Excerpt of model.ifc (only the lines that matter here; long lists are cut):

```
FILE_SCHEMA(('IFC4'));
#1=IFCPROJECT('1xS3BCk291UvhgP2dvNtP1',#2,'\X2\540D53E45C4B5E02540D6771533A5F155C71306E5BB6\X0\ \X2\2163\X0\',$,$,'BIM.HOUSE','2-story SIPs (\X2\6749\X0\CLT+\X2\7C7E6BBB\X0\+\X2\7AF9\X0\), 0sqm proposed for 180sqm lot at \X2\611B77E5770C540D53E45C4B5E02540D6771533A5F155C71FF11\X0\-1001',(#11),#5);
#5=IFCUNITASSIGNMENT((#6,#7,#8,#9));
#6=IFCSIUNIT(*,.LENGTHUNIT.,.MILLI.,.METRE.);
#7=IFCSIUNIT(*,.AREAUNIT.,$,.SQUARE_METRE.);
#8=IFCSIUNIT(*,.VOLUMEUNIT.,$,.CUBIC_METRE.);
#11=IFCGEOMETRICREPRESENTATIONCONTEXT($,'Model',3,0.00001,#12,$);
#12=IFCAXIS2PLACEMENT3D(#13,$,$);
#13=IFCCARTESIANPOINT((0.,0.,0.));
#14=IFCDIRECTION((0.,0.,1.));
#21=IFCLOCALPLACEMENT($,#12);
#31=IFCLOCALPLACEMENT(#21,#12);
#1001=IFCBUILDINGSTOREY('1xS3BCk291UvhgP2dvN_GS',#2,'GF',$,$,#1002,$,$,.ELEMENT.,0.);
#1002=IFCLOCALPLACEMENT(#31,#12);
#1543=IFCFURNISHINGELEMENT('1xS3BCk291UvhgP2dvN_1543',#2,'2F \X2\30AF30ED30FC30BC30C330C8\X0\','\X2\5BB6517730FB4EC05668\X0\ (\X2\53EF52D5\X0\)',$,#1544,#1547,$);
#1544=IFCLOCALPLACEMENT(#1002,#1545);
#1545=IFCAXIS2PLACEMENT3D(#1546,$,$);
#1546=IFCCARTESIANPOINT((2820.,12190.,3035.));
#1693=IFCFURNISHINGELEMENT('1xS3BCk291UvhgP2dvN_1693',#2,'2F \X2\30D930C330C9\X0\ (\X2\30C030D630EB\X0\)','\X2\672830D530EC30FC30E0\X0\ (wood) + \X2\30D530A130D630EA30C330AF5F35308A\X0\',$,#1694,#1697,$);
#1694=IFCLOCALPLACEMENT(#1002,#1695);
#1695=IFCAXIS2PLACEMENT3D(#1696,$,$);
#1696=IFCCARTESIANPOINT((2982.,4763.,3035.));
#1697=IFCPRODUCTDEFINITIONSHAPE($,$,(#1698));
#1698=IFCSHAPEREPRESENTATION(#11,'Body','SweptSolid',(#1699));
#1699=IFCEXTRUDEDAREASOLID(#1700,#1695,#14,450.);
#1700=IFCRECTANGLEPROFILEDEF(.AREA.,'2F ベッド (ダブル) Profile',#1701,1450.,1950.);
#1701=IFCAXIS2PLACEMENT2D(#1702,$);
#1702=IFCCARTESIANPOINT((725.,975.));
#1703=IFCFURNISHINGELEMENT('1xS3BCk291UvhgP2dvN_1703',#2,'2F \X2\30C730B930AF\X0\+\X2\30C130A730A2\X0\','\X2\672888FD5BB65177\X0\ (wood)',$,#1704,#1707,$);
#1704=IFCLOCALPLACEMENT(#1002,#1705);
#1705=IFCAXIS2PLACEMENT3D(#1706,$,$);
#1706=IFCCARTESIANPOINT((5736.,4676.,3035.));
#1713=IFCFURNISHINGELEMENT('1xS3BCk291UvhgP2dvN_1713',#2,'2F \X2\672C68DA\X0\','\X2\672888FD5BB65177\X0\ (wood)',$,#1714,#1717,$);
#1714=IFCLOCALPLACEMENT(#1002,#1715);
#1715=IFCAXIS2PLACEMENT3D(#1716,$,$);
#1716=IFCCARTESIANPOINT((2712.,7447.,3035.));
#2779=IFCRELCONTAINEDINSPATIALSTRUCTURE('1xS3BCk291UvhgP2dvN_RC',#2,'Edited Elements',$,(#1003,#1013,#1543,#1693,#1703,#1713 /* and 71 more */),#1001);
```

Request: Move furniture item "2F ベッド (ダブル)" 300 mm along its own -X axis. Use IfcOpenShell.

```python
import ifcopenshell
import ifcopenshell.api.geometry
import ifcopenshell.util.placement

model = ifcopenshell.open("model.ifc")

item = model.by_guid("1xS3BCk291UvhgP2dvN_1693")
matrix = ifcopenshell.util.placement.get_local_placement(item.ObjectPlacement)
matrix[:3, 3] -= matrix[:3, 0] * 300.0
ifcopenshell.api.geometry.edit_object_placement(model, product=item, matrix=matrix, is_si=False)

print(ifcopenshell.util.placement.get_local_placement(item.ObjectPlacement).round(3) + 0.0)

model.write("model_updated.ifc")
```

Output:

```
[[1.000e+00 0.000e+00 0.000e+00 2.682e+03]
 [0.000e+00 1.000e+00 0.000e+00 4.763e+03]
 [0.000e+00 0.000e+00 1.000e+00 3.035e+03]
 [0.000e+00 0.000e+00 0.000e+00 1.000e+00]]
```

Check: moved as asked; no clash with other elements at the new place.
